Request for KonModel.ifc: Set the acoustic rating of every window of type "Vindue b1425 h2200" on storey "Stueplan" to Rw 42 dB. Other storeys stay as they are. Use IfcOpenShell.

First a look at what the model holds.

```python
import ifcopenshell
import ifcopenshell.util.element

model = ifcopenshell.open("KonModel.ifc")
print(model.schema)
storey = next(s for s in model.by_type("IfcBuildingStorey") if s.Name == "Stueplan")
windows = [e for e in ifcopenshell.util.element.get_decomposition(storey) if e.is_a("IfcWindow")]
seen = {}
for e in windows:
    element_type = ifcopenshell.util.element.get_type(e)
    key = (element_type.Name if element_type != e and element_type else None, ifcopenshell.util.element.get_pset(e, "Pset_WindowCommon", "AcousticRating"))
    seen[key] = seen.get(key, 0) + 1
for (name, value), count in sorted(seen.items(), key=str):
    print(count, "x", name, "|", value)
```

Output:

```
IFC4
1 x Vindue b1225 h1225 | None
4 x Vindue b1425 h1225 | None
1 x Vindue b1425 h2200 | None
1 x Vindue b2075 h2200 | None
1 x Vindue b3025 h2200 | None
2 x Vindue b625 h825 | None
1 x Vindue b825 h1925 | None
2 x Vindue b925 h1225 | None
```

```python
import ifcopenshell
import ifcopenshell.api.pset
import ifcopenshell.util.element

model = ifcopenshell.open("KonModel.ifc")

storey = next(s for s in model.by_type("IfcBuildingStorey") if s.Name == "Stueplan")
windows = [e for e in ifcopenshell.util.element.get_decomposition(storey) if e.is_a("IfcWindow")]

count = 0
for e in windows:
    element_type = ifcopenshell.util.element.get_type(e)
    if element_type in (None, e) or element_type.Name != "Vindue b1425 h2200":
        continue
    # add_pset returns the element's existing set when there is one.
    pset = ifcopenshell.api.pset.add_pset(model, product=e, name="Pset_WindowCommon")
    ifcopenshell.api.pset.edit_pset(model, pset=pset, properties={"AcousticRating": "Rw 42 dB"})
    count += 1

print(count, "windows updated")

model.write("KonModel_updated.ifc")
```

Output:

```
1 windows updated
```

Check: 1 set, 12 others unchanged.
